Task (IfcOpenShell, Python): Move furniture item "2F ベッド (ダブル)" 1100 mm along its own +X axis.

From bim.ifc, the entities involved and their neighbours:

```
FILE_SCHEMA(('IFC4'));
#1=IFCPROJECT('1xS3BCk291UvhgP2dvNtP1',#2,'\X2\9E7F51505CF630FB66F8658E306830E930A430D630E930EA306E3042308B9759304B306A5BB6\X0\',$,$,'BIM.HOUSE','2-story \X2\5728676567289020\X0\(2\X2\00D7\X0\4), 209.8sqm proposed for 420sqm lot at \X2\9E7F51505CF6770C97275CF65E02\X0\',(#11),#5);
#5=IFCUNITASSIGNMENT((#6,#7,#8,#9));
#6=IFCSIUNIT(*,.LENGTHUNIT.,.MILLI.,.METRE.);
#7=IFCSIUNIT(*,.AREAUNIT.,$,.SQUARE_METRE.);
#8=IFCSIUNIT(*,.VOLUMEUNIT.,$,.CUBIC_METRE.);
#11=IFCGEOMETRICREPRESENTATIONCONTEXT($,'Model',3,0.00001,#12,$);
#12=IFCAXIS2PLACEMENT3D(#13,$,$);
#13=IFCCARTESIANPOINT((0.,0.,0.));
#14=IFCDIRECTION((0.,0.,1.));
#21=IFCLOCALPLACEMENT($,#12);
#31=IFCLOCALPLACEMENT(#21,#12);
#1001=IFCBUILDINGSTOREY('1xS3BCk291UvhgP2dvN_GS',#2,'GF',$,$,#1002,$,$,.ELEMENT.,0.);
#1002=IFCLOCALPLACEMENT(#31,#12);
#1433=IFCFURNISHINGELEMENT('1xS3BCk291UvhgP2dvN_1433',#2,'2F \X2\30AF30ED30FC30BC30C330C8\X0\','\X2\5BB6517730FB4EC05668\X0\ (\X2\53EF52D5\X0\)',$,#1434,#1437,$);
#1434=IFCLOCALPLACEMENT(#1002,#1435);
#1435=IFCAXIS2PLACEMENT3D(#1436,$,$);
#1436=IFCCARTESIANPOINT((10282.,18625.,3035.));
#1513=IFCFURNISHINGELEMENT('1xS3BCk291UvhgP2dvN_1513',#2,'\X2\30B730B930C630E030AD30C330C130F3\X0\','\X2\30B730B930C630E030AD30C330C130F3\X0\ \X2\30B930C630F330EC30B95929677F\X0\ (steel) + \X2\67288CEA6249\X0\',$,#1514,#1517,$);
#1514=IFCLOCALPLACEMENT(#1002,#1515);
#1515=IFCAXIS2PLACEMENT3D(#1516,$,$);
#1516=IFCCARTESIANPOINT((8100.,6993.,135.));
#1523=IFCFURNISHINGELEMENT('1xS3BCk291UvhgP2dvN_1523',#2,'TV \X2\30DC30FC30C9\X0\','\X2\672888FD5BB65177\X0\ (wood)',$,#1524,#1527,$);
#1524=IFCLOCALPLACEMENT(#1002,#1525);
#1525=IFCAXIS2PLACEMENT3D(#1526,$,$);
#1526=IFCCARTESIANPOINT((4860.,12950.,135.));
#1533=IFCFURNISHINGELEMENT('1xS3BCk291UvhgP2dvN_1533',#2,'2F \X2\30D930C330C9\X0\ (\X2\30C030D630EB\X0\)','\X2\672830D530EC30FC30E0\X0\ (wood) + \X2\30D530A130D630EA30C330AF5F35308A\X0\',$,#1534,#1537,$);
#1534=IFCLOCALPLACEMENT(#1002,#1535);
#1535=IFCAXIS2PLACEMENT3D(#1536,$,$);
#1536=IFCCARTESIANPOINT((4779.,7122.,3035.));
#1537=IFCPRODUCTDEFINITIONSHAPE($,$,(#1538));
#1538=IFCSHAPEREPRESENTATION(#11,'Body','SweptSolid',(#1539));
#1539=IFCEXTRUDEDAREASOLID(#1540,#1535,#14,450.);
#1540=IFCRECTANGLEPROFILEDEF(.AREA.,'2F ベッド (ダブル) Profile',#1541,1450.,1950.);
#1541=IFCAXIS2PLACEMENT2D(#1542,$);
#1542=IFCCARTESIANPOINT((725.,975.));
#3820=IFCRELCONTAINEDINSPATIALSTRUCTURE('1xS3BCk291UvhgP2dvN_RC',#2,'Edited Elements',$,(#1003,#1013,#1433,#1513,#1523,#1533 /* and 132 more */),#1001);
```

```python
import ifcopenshell
import ifcopenshell.api.geometry
import ifcopenshell.util.placement

model = ifcopenshell.open("bim.ifc")

item = model.by_guid("1xS3BCk291UvhgP2dvN_1533")
matrix = ifcopenshell.util.placement.get_local_placement(item.ObjectPlacement)
matrix[:3, 3] += matrix[:3, 0] * 1100.0
ifcopenshell.api.geometry.edit_object_placement(model, product=item, matrix=matrix, is_si=False)

print(ifcopenshell.util.placement.get_local_placement(item.ObjectPlacement).round(3) + 0.0)

model.write("bim_edited.ifc")
```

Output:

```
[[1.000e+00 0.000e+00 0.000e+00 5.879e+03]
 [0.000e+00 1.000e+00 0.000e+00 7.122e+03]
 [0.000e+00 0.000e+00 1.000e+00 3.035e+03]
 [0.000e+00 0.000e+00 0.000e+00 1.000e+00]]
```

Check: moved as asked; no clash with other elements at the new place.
